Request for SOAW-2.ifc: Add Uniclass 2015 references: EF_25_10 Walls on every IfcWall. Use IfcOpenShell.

First a look at what the model holds.

```python
import ifcopenshell

model = ifcopenshell.open("SOAW-2.ifc")
print(model.schema)
print("classifications:", [c.Name for c in model.by_type("IfcClassification")])
for ifc_class in ("IfcDoor", "IfcRoof", "IfcStair", "IfcWall", "IfcWindow"):
    print(ifc_class, len(model.by_type(ifc_class)))
```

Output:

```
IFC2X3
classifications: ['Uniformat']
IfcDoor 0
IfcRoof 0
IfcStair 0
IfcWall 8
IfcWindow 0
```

```python
import ifcopenshell
import ifcopenshell.api.classification

model = ifcopenshell.open("SOAW-2.ifc")

# IFC2X3 requires Source and Edition and has no link from the project to the system.
system = model.create_entity("IfcClassification", Source="NBS", Edition="2015", Name="Uniclass 2015")

codes = {
    "IfcWall": ("EF_25_10", "Walls"),
}
for ifc_class, (code, name) in codes.items():
    products = model.by_type(ifc_class)
    ifcopenshell.api.classification.add_reference(
        model, products=products, classification=system, identification=code, name=name
    )
    print(code, len(products))

model.write("SOAW-2_edited.ifc")
```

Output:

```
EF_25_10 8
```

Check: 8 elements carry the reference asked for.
